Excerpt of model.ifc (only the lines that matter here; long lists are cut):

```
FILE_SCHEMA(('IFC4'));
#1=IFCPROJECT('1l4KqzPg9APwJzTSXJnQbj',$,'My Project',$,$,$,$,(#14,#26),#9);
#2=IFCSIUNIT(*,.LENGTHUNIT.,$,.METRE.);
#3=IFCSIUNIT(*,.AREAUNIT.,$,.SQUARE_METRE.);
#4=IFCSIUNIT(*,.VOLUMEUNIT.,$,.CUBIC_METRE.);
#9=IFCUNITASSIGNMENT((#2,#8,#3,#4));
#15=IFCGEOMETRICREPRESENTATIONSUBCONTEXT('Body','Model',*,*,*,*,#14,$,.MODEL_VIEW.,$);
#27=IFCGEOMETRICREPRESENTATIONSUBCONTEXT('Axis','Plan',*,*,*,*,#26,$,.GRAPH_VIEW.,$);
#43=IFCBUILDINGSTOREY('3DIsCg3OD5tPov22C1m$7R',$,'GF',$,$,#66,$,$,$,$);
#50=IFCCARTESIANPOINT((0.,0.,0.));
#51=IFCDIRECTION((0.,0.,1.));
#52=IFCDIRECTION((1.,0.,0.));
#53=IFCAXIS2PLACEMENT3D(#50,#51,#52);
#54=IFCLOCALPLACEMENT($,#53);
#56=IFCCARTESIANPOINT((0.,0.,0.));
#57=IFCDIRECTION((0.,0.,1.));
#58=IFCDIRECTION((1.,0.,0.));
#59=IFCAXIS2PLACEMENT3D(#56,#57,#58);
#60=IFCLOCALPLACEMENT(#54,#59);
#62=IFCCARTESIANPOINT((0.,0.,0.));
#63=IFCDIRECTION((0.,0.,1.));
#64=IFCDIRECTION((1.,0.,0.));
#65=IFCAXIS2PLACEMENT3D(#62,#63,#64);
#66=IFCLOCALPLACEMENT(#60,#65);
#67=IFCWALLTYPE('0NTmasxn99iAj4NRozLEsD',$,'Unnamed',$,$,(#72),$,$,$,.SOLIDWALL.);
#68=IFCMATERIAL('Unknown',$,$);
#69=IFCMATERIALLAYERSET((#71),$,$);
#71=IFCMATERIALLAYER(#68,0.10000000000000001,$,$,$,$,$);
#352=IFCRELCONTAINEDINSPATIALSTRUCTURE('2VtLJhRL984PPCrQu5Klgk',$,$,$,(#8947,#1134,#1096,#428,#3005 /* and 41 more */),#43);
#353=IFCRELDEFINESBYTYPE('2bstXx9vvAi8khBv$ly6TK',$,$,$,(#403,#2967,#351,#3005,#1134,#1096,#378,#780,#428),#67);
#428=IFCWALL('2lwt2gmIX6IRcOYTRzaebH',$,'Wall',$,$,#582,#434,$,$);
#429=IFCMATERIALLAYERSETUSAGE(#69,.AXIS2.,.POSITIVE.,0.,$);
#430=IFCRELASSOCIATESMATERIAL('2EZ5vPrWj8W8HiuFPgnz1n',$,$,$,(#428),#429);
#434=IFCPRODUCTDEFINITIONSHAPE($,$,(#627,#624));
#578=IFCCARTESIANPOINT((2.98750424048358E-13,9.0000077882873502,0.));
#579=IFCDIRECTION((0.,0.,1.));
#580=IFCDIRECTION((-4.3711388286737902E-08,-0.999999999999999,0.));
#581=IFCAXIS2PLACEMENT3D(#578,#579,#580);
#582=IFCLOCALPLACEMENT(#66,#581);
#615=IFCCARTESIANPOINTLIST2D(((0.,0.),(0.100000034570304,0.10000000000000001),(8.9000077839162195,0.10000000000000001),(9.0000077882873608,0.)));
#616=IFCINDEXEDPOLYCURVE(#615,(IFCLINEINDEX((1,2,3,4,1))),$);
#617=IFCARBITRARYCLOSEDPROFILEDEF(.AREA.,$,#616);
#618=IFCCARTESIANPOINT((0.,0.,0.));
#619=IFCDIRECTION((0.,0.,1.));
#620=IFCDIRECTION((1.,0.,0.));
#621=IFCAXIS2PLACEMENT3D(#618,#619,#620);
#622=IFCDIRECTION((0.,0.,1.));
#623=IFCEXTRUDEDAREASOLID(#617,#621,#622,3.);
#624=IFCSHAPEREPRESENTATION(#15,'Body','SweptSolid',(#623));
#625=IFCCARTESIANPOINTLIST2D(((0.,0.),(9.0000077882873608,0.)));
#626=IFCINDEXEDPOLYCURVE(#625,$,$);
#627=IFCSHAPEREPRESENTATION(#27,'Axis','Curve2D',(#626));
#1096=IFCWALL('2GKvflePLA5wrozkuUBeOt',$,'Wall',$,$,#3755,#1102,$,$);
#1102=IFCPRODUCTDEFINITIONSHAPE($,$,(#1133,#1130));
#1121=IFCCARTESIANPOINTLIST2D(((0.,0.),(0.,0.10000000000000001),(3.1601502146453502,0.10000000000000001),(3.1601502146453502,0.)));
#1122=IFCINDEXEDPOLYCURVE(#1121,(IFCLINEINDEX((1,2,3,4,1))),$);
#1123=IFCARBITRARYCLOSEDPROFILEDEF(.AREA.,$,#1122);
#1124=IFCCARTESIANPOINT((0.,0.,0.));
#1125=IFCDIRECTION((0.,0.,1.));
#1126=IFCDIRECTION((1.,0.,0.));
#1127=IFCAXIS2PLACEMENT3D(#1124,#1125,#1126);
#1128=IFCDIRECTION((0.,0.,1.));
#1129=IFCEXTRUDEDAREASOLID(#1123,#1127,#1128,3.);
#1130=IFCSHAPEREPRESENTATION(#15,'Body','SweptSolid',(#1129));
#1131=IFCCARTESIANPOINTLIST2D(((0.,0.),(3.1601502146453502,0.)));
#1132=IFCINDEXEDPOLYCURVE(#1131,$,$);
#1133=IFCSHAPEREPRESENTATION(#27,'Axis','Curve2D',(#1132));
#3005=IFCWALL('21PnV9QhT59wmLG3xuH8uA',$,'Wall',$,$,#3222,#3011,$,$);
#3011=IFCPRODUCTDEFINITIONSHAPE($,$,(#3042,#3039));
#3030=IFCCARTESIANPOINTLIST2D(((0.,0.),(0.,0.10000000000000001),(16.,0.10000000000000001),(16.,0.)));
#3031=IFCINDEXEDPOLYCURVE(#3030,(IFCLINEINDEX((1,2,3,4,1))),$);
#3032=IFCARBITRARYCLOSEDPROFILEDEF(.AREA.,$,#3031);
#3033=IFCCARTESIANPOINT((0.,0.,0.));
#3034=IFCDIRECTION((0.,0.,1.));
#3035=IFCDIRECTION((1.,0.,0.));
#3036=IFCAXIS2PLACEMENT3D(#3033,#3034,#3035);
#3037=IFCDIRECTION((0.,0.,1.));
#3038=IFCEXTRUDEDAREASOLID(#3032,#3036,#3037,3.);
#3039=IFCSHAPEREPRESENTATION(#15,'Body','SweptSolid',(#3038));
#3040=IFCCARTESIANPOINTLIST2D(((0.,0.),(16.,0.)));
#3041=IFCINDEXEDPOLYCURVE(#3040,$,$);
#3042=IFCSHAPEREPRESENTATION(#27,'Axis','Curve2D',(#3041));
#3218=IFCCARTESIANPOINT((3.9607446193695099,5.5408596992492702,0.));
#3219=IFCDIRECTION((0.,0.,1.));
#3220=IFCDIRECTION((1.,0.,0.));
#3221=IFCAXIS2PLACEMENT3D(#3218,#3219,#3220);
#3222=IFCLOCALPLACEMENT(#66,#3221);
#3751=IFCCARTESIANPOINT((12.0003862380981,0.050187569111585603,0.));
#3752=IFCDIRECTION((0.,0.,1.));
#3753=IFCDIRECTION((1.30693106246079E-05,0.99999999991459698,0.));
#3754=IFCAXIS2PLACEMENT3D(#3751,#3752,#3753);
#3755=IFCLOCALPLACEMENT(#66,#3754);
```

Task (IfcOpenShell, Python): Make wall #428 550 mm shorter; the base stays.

```python
import ifcopenshell
import ifcopenshell.geom
import ifcopenshell.util.representation
import ifcopenshell.util.shape
import ifcopenshell.util.unit

model = ifcopenshell.open("model.ifc")
unit_scale = ifcopenshell.util.unit.calculate_unit_scale(model)
settings = ifcopenshell.geom.settings()


def volume(element):
    """Net volume in cubic metres, openings subtracted."""
    shape = ifcopenshell.geom.create_shape(settings, element)
    return ifcopenshell.util.shape.get_volume(shape.geometry)


wall = model.by_guid("2lwt2gmIX6IRcOYTRzaebH")
before = volume(wall)

body = ifcopenshell.util.representation.get_representation(wall, "Model", "Body")
solid = body.Items[0]
old_height = solid.Depth
solid.Depth -= 0.55 / unit_scale
after = volume(wall)

print(f"height {old_height:g} -> {solid.Depth:g}, volume {before:.3f} -> {after:.3f} m3")

model.write("model_rev.ifc")
```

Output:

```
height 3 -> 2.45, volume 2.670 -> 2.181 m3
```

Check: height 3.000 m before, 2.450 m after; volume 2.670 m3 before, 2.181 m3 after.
